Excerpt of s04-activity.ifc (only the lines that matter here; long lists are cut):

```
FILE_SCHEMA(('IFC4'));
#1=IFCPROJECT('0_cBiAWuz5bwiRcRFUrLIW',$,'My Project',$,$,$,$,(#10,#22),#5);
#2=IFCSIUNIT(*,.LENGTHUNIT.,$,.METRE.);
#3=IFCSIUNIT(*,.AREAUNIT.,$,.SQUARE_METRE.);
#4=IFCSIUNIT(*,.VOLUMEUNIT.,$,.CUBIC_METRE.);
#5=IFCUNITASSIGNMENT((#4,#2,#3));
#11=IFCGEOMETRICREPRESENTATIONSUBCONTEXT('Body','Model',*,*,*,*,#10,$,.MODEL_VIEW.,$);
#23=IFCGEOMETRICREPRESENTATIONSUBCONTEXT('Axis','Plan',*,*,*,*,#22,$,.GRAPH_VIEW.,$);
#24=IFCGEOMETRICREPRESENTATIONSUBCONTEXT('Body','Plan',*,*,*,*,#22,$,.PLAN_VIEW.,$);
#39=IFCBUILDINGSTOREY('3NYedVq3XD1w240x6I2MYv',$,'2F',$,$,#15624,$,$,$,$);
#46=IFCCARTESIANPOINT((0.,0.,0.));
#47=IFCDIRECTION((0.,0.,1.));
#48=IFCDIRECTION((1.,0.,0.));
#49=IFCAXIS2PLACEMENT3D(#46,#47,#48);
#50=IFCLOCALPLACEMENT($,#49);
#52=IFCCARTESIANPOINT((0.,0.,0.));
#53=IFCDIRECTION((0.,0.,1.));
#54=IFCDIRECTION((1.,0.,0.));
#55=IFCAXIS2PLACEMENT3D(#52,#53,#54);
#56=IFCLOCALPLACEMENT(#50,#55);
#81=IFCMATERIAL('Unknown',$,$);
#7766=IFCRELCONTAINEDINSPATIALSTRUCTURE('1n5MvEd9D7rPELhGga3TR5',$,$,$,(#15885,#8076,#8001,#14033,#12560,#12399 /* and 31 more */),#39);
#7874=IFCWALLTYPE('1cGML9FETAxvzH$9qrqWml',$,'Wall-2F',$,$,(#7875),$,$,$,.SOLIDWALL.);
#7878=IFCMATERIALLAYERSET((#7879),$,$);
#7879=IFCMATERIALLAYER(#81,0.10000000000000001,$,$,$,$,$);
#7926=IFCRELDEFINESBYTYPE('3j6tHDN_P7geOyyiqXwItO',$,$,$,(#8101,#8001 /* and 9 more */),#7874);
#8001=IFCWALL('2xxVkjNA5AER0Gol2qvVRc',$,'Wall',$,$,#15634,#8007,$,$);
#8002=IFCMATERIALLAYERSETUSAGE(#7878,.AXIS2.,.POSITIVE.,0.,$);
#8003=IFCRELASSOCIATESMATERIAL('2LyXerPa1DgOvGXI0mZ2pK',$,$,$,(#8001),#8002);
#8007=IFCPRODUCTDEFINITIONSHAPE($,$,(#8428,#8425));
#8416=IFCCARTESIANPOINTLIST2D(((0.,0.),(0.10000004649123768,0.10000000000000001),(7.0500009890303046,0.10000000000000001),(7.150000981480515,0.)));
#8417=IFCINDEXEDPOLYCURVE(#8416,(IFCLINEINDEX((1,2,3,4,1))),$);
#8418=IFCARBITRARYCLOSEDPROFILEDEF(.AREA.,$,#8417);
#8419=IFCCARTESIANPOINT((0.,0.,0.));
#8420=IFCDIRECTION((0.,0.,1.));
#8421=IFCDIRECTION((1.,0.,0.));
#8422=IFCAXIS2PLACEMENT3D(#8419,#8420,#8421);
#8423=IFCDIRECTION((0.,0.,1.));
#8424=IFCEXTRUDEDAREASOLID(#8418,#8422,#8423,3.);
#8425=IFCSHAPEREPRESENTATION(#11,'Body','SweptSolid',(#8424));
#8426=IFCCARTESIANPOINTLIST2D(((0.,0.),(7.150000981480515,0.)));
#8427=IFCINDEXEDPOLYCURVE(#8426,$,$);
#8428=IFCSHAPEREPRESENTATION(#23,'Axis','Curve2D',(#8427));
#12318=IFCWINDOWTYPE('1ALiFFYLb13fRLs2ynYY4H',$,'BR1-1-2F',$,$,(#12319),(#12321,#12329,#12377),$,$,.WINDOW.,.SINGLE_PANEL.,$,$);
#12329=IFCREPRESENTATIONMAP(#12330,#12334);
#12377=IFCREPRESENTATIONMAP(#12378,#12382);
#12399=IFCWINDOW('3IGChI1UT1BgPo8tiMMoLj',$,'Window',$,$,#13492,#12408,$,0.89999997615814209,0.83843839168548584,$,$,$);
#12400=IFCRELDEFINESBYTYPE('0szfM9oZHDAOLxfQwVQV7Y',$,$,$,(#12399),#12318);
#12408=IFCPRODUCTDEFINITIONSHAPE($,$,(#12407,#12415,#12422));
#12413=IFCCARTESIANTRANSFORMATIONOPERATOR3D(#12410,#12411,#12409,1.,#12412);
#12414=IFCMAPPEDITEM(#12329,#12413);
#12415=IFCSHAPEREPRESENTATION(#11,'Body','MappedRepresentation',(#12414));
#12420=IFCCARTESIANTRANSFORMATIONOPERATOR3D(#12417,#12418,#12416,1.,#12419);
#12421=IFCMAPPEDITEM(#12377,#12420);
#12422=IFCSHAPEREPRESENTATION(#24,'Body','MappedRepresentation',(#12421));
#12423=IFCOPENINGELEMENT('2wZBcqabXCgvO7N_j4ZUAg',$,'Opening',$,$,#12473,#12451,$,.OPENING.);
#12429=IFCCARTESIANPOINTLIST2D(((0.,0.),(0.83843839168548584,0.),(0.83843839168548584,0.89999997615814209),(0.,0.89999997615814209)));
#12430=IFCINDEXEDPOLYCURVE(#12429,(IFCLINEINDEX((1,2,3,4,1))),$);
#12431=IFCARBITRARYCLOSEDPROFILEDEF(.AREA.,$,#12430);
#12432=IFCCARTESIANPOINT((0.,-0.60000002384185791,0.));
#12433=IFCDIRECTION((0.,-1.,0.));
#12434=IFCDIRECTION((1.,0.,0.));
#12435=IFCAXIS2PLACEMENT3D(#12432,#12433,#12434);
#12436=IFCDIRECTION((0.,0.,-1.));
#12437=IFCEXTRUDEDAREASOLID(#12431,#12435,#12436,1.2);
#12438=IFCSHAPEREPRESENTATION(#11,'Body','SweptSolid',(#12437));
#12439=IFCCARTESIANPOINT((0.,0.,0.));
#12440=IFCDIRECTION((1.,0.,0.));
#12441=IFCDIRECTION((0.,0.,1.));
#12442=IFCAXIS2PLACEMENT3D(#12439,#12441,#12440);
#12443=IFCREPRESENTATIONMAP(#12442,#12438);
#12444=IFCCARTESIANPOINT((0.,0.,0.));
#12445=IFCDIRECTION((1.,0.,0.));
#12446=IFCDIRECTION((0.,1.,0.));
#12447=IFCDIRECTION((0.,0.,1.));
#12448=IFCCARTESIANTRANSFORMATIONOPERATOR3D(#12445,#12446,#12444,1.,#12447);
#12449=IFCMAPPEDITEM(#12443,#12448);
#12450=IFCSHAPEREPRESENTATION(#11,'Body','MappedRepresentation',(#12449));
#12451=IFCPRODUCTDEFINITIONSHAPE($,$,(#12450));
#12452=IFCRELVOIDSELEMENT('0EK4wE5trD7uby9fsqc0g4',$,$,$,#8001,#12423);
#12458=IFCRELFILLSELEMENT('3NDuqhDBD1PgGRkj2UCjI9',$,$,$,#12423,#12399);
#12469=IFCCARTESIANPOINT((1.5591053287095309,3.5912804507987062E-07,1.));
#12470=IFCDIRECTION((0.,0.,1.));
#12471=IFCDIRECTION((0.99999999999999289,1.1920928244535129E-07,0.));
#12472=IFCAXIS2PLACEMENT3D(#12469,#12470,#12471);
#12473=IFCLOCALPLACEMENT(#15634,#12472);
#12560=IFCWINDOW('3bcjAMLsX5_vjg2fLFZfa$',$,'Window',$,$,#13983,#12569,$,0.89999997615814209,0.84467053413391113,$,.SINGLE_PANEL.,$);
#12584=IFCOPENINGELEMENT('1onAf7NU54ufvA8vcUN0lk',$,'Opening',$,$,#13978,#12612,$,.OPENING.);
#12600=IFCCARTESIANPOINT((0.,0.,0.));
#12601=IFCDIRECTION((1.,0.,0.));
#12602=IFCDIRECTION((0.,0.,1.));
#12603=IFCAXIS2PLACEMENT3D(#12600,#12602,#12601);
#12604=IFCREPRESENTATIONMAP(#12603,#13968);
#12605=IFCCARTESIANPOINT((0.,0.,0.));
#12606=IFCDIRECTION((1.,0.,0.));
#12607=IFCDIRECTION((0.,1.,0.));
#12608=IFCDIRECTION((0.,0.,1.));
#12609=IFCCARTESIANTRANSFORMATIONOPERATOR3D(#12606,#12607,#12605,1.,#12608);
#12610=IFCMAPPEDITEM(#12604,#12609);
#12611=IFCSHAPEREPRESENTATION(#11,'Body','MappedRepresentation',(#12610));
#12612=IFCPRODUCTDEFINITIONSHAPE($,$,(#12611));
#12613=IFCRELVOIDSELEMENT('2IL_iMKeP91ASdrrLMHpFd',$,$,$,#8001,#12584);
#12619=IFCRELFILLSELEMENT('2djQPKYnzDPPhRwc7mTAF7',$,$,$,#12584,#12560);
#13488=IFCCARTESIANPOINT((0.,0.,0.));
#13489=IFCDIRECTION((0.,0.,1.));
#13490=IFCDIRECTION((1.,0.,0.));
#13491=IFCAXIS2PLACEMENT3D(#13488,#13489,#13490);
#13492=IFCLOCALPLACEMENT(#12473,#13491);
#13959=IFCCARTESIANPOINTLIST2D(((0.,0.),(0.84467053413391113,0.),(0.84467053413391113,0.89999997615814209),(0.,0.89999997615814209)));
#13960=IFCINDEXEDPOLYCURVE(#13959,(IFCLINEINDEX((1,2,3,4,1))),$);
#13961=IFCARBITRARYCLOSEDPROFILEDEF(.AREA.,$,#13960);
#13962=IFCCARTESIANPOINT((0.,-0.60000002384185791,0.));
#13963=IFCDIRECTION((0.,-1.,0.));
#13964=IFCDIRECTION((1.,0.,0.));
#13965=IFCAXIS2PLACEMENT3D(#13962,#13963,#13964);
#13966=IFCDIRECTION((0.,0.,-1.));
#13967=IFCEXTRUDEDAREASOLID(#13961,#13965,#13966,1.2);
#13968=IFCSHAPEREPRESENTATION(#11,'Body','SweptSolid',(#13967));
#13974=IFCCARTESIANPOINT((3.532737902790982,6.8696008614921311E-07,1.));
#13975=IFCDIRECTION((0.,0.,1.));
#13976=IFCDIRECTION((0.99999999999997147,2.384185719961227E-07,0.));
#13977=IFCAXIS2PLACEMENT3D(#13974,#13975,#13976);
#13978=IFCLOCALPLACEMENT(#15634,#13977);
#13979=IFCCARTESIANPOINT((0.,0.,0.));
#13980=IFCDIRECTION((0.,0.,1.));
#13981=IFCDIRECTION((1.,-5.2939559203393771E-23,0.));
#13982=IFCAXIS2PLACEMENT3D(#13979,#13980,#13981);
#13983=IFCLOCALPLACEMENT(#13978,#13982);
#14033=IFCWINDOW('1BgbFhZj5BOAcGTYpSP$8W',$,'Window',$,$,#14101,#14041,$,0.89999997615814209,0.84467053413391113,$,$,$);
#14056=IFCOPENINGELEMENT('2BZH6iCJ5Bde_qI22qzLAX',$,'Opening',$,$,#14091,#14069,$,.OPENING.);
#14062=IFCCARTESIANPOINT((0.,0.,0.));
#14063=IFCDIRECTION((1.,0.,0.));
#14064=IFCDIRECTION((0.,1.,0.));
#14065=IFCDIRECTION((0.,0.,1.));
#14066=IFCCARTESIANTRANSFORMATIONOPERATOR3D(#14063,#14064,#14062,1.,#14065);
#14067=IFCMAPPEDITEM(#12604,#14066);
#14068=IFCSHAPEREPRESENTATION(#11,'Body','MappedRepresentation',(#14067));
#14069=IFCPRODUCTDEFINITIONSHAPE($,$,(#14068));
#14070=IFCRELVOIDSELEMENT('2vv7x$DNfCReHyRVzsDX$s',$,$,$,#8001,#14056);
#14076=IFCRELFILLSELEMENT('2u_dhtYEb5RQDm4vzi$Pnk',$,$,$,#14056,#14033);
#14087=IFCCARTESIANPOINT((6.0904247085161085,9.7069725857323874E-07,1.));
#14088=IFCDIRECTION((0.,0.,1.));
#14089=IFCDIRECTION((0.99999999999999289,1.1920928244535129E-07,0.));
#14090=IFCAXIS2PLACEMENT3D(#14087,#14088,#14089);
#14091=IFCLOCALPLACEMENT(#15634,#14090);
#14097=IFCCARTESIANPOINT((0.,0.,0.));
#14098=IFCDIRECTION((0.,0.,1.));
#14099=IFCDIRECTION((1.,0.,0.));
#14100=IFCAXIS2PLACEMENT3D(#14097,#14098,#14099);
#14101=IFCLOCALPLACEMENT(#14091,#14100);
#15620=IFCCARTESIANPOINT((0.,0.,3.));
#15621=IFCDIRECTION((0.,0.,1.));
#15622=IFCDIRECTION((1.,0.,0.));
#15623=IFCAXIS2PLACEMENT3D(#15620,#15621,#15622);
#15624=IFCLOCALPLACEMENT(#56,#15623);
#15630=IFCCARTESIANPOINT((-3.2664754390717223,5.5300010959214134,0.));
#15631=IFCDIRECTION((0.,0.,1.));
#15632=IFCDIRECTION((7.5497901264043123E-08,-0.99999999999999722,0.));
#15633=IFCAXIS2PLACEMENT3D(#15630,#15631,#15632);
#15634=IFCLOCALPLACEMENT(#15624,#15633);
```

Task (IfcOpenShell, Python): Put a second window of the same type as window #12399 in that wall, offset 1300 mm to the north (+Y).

```python
import ifcopenshell
import ifcopenshell.api.feature
import ifcopenshell.api.geometry
import ifcopenshell.api.root
import ifcopenshell.geom
import ifcopenshell.util.element
import ifcopenshell.util.placement
import ifcopenshell.util.shape
import ifcopenshell.util.unit

model = ifcopenshell.open("s04-activity.ifc")
unit_scale = ifcopenshell.util.unit.calculate_unit_scale(model)
settings = ifcopenshell.geom.settings()


def volume(element):
    """Net volume in cubic metres, openings subtracted."""
    shape = ifcopenshell.geom.create_shape(settings, element)
    return ifcopenshell.util.shape.get_volume(shape.geometry)


window = model.by_id(12399)
opening = window.FillsVoids[0].RelatingOpeningElement
wall = opening.VoidsElements[0].RelatingBuildingElement
before = volume(wall)
shift = ifcopenshell.util.placement.get_local_placement(wall.ObjectPlacement)[:3, 0] * -1.3 / unit_scale

# copy_class copies the void relationship, type, container and properties, but no geometry.
new_opening = ifcopenshell.api.root.copy_class(model, product=opening)
new_opening.Representation = ifcopenshell.util.element.copy_deep(
    model, opening.Representation, exclude=["IfcGeometricRepresentationContext", "IfcRepresentationMap"]
)
new_window = ifcopenshell.api.root.copy_class(model, product=window)
new_window.Representation = ifcopenshell.util.element.copy_deep(
    model, window.Representation, exclude=["IfcGeometricRepresentationContext", "IfcRepresentationMap"]
)
ifcopenshell.api.feature.add_filling(model, opening=new_opening, element=new_window)

for old, new in ((opening, new_opening), (window, new_window)):
    matrix = ifcopenshell.util.placement.get_local_placement(old.ObjectPlacement)
    matrix[:3, 3] += shift
    ifcopenshell.api.geometry.edit_object_placement(model, product=new, matrix=matrix, is_si=False)

after = volume(wall)

print(f"wall volume {before:.3f} -> {after:.3f} m3")

model.write("s04-activity_v2.ifc")
```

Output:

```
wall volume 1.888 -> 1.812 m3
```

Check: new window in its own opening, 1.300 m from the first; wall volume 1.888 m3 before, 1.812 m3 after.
